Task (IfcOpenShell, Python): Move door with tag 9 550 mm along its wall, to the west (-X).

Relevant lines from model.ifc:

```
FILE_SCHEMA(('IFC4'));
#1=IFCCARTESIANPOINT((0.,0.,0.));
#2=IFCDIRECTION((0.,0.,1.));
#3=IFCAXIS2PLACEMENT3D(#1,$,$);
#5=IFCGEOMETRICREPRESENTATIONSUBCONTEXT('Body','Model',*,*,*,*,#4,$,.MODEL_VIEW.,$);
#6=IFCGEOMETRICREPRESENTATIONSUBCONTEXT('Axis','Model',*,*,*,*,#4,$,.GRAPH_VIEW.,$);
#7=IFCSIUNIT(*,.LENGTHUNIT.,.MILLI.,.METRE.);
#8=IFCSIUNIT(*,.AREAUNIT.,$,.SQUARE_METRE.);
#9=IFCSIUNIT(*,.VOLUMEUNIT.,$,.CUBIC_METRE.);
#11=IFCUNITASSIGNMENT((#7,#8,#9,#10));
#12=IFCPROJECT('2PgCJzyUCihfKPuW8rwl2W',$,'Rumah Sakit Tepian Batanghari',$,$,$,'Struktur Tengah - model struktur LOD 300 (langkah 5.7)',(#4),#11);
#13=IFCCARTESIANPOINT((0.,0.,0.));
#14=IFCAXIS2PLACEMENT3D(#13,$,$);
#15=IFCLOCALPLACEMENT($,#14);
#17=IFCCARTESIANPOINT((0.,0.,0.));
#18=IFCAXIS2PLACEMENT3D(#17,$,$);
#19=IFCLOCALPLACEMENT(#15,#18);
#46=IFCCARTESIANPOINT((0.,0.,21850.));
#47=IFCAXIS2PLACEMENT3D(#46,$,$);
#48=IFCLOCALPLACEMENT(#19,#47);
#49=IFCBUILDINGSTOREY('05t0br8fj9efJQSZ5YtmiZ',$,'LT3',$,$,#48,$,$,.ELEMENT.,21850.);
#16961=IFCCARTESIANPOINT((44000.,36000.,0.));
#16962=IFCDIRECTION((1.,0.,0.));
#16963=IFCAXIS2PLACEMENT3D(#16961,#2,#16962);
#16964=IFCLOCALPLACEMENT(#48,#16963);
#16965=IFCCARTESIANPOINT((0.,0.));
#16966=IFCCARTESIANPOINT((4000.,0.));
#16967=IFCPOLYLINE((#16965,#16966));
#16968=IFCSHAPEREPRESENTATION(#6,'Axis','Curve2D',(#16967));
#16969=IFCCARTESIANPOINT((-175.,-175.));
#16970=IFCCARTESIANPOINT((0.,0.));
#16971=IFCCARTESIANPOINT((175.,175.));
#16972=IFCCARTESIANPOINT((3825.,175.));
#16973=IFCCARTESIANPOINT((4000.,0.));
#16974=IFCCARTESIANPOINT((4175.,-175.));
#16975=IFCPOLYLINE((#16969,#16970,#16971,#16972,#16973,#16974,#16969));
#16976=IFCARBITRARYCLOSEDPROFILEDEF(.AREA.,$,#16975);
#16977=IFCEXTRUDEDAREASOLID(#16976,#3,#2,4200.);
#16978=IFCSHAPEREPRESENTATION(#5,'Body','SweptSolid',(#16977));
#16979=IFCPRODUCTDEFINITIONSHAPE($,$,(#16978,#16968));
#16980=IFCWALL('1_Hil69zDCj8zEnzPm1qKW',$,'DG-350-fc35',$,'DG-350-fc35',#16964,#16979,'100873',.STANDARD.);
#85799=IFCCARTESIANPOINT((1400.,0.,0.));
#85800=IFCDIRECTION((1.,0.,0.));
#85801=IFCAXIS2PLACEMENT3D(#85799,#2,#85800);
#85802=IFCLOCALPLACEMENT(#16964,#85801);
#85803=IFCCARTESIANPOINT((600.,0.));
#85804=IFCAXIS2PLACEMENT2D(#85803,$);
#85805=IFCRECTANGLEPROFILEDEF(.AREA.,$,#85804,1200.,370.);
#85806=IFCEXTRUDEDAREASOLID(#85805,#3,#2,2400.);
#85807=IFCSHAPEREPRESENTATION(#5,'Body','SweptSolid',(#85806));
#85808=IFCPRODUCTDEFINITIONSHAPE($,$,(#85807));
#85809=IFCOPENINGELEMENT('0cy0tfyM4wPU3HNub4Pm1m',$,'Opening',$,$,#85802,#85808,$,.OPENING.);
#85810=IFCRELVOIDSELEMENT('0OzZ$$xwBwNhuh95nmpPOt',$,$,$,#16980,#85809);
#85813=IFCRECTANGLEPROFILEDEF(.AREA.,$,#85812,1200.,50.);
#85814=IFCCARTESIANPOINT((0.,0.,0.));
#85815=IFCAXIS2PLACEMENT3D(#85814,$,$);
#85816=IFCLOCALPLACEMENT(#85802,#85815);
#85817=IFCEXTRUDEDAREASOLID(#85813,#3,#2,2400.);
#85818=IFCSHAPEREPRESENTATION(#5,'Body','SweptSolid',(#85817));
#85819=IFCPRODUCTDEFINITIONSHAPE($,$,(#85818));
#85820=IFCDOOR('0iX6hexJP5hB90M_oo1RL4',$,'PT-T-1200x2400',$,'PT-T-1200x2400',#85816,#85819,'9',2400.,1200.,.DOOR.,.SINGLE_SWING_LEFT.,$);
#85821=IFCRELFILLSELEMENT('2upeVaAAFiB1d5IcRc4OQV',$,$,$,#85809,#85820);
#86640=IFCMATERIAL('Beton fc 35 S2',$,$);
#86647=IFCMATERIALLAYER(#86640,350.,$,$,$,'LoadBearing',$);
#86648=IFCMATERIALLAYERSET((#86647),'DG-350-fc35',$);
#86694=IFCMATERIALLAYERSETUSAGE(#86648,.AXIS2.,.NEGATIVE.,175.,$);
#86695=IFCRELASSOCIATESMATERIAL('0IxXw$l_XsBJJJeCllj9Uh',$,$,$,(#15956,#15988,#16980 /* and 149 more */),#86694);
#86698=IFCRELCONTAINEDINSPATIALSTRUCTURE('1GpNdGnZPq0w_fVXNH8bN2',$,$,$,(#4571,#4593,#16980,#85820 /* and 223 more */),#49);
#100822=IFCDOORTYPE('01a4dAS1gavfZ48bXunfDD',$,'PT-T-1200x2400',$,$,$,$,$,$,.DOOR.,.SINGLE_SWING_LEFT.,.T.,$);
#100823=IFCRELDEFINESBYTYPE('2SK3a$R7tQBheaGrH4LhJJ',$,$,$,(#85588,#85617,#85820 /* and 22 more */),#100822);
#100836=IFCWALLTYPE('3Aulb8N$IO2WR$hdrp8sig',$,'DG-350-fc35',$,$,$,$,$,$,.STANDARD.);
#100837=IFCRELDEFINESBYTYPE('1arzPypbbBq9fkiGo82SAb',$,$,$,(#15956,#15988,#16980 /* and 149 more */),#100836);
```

```python
import ifcopenshell
import ifcopenshell.api.geometry
import ifcopenshell.util.placement
import ifcopenshell.util.unit

model = ifcopenshell.open("model.ifc")
unit_scale = ifcopenshell.util.unit.calculate_unit_scale(model)

door = model.by_id(85820)
opening = door.FillsVoids[0].RelatingOpeningElement
wall = opening.VoidsElements[0].RelatingBuildingElement

wall_matrix = ifcopenshell.util.placement.get_local_placement(wall.ObjectPlacement)
shift = wall_matrix[:3, 0] * -0.55 / unit_scale
before = ifcopenshell.util.placement.get_local_placement(door.ObjectPlacement)[:3, 3].copy()

# The door is placed relative to its opening, so it follows when the opening moves.
matrix = ifcopenshell.util.placement.get_local_placement(opening.ObjectPlacement)
matrix[:3, 3] += shift
ifcopenshell.api.geometry.edit_object_placement(
    model, product=opening, matrix=matrix, is_si=False, should_transform_children=True
)

after = ifcopenshell.util.placement.get_local_placement(door.ObjectPlacement)[:3, 3]
print("door moved by", (after - before).round(3) + 0.0)

model.write("model-out.ifc")
```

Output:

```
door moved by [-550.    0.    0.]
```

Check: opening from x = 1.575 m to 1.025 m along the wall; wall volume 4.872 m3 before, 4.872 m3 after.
